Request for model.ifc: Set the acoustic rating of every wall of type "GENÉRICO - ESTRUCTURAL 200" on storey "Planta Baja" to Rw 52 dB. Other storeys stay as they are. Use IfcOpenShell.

First a look at what the model holds.

```python
import ifcopenshell
import ifcopenshell.util.element

model = ifcopenshell.open("model.ifc")
print(model.schema)
storey = next(s for s in model.by_type("IfcBuildingStorey") if s.Name == "Planta Baja")
walls = [e for e in ifcopenshell.util.element.get_decomposition(storey) if e.is_a("IfcWall")]
seen = {}
for e in walls:
    element_type = ifcopenshell.util.element.get_type(e)
    key = (element_type.Name if element_type != e and element_type else None, ifcopenshell.util.element.get_pset(e, "Pset_WallCommon", "AcousticRating"))
    seen[key] = seen.get(key, 0) + 1
for (name, value), count in sorted(seen.items(), key=str):
    print(count, "x", name, "|", value)
```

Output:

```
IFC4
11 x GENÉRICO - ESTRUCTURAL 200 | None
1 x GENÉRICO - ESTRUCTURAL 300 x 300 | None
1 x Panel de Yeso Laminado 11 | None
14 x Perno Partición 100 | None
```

```python
import ifcopenshell
import ifcopenshell.api.pset
import ifcopenshell.util.element

model = ifcopenshell.open("model.ifc")

storey = next(s for s in model.by_type("IfcBuildingStorey") if s.Name == "Planta Baja")
walls = [e for e in ifcopenshell.util.element.get_decomposition(storey) if e.is_a("IfcWall")]

count = 0
for e in walls:
    element_type = ifcopenshell.util.element.get_type(e)
    if element_type in (None, e) or element_type.Name != "GENÉRICO - ESTRUCTURAL 200":
        continue
    # add_pset returns the element's existing set when there is one.
    pset = ifcopenshell.api.pset.add_pset(model, product=e, name="Pset_WallCommon")
    ifcopenshell.api.pset.edit_pset(model, pset=pset, properties={"AcousticRating": "Rw 52 dB"})
    count += 1

print(count, "walls updated")

model.write("model_rev.ifc")
```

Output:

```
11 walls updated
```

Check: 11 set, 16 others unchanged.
